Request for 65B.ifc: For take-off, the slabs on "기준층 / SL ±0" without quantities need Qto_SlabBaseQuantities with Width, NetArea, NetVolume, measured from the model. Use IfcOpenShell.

First a look at what the model holds.

```python
import ifcopenshell
import ifcopenshell.util.element
import ifcopenshell.util.unit

model = ifcopenshell.open("65B.ifc")
print(model.schema)
for unit_type in ("LENGTHUNIT", "AREAUNIT", "VOLUMEUNIT"):
    print(unit_type, ifcopenshell.util.unit.calculate_unit_scale(model, unit_type))
storey = next(s for s in model.by_type("IfcBuildingStorey") if s.Name == "기준층 / SL ±0")
slabs = [e for e in ifcopenshell.util.element.get_decomposition(storey) if e.is_a("IfcSlab")]
for e in sorted(slabs, key=lambda e: e.id()):
    print(e.id(), e.is_a(), e.Name, list(ifcopenshell.util.element.get_psets(e, qtos_only=True)), sep=" | ")
```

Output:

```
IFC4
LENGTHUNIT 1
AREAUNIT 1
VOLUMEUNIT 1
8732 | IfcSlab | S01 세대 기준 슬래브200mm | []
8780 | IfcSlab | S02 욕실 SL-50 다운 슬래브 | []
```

```python
import ifcopenshell
import ifcopenshell.api.pset
import ifcopenshell.geom
import ifcopenshell.util.element
import ifcopenshell.util.shape
import ifcopenshell.util.unit

model = ifcopenshell.open("65B.ifc")
unit_scale = ifcopenshell.util.unit.calculate_unit_scale(model)
area_scale = ifcopenshell.util.unit.calculate_unit_scale(model, "AREAUNIT")
volume_scale = ifcopenshell.util.unit.calculate_unit_scale(model, "VOLUMEUNIT")
settings = ifcopenshell.geom.settings()

storey = next(s for s in model.by_type("IfcBuildingStorey") if s.Name == "기준층 / SL ±0")
slabs = [e for e in ifcopenshell.util.element.get_decomposition(storey) if e.is_a("IfcSlab")]

for e in sorted(slabs, key=lambda e: e.id()):
    if ifcopenshell.util.element.get_psets(e, qtos_only=True, should_inherit=False):
        continue
    # Geometry comes back in metres, in the element's own axes.
    shape = ifcopenshell.geom.create_shape(settings, e)
    values = {
        "Width": ifcopenshell.util.shape.get_z(shape.geometry) / unit_scale,
        "NetArea": ifcopenshell.util.shape.get_footprint_area(shape.geometry) / area_scale,
        "NetVolume": ifcopenshell.util.shape.get_volume(shape.geometry) / volume_scale,
    }
    qto = ifcopenshell.api.pset.add_qto(model, product=e, name="Qto_SlabBaseQuantities")
    ifcopenshell.api.pset.edit_qto(model, qto=qto, properties=values)
    print(e.id(), {k: round(v, 3) for k, v in values.items()})

model.write("65B_edited.ifc")
```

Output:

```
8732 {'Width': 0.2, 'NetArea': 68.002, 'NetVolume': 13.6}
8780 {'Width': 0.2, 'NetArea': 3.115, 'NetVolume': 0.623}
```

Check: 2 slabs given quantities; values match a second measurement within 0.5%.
